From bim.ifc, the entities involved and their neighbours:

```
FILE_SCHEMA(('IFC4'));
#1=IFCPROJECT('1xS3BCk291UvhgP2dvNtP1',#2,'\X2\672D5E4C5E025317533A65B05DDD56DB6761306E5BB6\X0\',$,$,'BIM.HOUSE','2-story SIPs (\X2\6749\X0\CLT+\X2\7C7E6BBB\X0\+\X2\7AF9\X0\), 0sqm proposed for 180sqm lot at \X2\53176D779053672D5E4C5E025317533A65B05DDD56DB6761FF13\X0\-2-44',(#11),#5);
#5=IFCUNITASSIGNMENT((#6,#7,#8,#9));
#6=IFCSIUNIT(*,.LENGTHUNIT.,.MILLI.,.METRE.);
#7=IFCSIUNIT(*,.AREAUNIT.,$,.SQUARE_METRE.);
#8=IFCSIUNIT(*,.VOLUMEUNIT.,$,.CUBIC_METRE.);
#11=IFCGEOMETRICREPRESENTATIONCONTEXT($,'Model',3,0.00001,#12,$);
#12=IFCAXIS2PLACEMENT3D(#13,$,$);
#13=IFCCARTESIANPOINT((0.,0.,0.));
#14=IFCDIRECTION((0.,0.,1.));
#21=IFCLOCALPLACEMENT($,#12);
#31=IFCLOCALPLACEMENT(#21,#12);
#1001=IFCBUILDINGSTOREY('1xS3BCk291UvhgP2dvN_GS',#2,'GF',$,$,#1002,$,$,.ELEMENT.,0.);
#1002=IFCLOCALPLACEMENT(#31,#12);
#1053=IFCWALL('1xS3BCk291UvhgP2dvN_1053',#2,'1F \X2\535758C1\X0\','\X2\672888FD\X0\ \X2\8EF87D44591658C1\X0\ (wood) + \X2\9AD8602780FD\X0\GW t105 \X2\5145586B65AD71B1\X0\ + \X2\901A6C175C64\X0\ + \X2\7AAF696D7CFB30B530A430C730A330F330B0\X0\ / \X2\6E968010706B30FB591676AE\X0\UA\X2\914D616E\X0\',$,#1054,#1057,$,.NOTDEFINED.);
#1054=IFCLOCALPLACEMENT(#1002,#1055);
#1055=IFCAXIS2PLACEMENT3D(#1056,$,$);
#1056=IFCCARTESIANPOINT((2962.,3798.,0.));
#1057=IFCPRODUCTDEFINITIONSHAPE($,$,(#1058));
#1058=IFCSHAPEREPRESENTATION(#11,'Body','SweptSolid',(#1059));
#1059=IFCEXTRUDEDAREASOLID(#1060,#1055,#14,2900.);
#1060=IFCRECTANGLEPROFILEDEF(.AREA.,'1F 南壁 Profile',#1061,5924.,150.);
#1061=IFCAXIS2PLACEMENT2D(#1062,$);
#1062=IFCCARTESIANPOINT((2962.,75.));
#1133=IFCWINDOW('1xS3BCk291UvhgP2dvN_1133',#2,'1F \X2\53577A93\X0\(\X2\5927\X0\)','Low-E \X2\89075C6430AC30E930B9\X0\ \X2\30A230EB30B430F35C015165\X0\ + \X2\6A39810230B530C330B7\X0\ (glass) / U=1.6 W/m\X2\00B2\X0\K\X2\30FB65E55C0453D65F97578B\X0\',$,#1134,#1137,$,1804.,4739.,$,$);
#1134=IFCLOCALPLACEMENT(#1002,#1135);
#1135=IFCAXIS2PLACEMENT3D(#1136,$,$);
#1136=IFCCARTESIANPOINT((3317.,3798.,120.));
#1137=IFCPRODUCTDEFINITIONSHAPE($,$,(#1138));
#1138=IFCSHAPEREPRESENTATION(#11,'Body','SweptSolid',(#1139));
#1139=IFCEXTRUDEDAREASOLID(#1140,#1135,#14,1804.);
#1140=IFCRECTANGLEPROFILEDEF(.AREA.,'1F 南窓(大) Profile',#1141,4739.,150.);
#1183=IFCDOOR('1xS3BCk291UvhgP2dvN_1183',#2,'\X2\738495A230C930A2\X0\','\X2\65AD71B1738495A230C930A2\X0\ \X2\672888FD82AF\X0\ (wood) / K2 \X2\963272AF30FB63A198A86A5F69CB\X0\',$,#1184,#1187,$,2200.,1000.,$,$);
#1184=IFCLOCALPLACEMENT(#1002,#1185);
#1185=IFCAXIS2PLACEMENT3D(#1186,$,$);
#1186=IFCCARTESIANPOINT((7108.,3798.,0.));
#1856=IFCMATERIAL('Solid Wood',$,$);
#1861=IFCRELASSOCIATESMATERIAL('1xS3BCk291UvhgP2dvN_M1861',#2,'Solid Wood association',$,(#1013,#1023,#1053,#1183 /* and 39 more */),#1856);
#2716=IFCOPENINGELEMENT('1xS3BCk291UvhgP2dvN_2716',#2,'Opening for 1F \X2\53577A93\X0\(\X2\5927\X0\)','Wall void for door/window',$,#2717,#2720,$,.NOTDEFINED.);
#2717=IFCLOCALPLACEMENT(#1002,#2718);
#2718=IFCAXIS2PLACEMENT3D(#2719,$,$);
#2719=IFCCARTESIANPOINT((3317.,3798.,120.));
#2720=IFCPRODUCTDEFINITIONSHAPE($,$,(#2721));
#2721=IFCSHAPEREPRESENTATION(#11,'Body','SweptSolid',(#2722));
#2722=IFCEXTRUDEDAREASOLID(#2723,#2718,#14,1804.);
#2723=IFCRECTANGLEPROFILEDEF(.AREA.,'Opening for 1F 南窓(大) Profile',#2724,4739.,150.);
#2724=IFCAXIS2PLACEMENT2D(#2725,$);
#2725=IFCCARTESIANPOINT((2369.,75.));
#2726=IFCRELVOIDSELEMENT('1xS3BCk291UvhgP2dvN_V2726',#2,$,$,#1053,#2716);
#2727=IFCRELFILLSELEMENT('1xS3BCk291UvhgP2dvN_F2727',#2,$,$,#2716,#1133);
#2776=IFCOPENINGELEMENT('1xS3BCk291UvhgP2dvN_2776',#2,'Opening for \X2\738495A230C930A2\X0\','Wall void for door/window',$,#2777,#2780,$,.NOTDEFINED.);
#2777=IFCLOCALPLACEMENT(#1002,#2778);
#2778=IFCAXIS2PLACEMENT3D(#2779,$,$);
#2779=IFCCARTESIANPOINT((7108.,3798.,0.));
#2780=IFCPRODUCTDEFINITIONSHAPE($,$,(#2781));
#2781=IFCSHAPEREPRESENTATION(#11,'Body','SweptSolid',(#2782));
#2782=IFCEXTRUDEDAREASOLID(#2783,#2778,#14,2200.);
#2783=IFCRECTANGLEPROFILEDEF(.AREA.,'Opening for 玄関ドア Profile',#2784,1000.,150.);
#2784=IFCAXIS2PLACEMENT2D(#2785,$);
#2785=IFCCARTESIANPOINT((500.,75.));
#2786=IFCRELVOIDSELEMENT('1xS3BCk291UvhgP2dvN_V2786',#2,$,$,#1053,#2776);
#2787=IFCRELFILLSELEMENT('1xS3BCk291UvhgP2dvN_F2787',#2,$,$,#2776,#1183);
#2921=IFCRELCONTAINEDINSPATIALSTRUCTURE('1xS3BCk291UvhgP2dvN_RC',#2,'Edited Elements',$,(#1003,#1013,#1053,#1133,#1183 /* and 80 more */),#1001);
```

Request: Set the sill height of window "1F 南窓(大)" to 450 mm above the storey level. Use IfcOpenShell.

```python
import numpy as np
import ifcopenshell
import ifcopenshell.api.geometry
import ifcopenshell.geom
import ifcopenshell.util.element
import ifcopenshell.util.placement
import ifcopenshell.util.shape
import ifcopenshell.util.unit

model = ifcopenshell.open("bim.ifc")
unit_scale = ifcopenshell.util.unit.calculate_unit_scale(model)

window = model.by_id(1133)
opening = window.FillsVoids[0].RelatingOpeningElement
storey = ifcopenshell.util.element.get_container(window, ifc_class="IfcBuildingStorey")
level = ifcopenshell.util.placement.get_local_placement(storey.ObjectPlacement)[2, 3]

# The opening's origin need not be at the sill, so measure its lowest point.
shape = ifcopenshell.geom.create_shape(ifcopenshell.geom.settings(), opening)
bottom = ifcopenshell.util.shape.get_shape_bottom_elevation(shape, shape.geometry) / unit_scale
dz = level + 450.0 - bottom

shift = np.array([0.0, 0.0, dz])
# The window is not placed relative to its opening, so move both.
for product in (opening, window):
    matrix = ifcopenshell.util.placement.get_local_placement(product.ObjectPlacement)
    matrix[:3, 3] += shift
    ifcopenshell.api.geometry.edit_object_placement(model, product=product, matrix=matrix, is_si=False)

print(f"moved by {dz * unit_scale:+.3f} m")

model.write("bim-out.ifc")
```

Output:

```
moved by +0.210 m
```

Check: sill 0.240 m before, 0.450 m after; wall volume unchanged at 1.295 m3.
